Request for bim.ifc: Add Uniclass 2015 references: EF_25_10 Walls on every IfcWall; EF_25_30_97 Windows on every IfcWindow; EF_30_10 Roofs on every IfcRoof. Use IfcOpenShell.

First a look at what the model holds.

```python
import ifcopenshell

model = ifcopenshell.open("bim.ifc")
print(model.schema)
print("classifications:", [c.Name for c in model.by_type("IfcClassification")])
for ifc_class in ("IfcDoor", "IfcRoof", "IfcStair", "IfcWall", "IfcWindow"):
    print(ifc_class, len(model.by_type(ifc_class)))
```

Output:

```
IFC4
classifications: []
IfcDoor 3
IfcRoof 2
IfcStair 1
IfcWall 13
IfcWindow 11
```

```python
import ifcopenshell
import ifcopenshell.api.classification

model = ifcopenshell.open("bim.ifc")

system = ifcopenshell.api.classification.add_classification(model, classification="Uniclass 2015")

codes = {
    "IfcWall": ("EF_25_10", "Walls"),
    "IfcWindow": ("EF_25_30_97", "Windows"),
    "IfcRoof": ("EF_30_10", "Roofs"),
}
for ifc_class, (code, name) in codes.items():
    products = model.by_type(ifc_class)
    ifcopenshell.api.classification.add_reference(
        model, products=products, classification=system, identification=code, name=name
    )
    print(code, len(products))

model.write("bim_v2.ifc")
```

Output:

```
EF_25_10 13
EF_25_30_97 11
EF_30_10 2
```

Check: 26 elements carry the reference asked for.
